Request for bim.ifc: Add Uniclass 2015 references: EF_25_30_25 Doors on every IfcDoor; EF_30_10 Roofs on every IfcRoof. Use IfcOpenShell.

First a look at what the model holds.

```python
import ifcopenshell

model = ifcopenshell.open("bim.ifc")
print(model.schema)
print("classifications:", [c.Name for c in model.by_type("IfcClassification")])
for ifc_class in ("IfcDoor", "IfcRoof", "IfcStair", "IfcWall", "IfcWindow"):
    print(ifc_class, len(model.by_type(ifc_class)))
```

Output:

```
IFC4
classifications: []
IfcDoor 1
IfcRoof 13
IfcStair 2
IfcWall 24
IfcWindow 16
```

```python
import ifcopenshell
import ifcopenshell.api.classification

model = ifcopenshell.open("bim.ifc")

system = ifcopenshell.api.classification.add_classification(model, classification="Uniclass 2015")

codes = {
    "IfcDoor": ("EF_25_30_25", "Doors"),
    "IfcRoof": ("EF_30_10", "Roofs"),
}
for ifc_class, (code, name) in codes.items():
    products = model.by_type(ifc_class)
    ifcopenshell.api.classification.add_reference(
        model, products=products, classification=system, identification=code, name=name
    )
    print(code, len(products))

model.write("bim-out.ifc")
```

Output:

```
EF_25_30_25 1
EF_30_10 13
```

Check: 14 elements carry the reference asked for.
